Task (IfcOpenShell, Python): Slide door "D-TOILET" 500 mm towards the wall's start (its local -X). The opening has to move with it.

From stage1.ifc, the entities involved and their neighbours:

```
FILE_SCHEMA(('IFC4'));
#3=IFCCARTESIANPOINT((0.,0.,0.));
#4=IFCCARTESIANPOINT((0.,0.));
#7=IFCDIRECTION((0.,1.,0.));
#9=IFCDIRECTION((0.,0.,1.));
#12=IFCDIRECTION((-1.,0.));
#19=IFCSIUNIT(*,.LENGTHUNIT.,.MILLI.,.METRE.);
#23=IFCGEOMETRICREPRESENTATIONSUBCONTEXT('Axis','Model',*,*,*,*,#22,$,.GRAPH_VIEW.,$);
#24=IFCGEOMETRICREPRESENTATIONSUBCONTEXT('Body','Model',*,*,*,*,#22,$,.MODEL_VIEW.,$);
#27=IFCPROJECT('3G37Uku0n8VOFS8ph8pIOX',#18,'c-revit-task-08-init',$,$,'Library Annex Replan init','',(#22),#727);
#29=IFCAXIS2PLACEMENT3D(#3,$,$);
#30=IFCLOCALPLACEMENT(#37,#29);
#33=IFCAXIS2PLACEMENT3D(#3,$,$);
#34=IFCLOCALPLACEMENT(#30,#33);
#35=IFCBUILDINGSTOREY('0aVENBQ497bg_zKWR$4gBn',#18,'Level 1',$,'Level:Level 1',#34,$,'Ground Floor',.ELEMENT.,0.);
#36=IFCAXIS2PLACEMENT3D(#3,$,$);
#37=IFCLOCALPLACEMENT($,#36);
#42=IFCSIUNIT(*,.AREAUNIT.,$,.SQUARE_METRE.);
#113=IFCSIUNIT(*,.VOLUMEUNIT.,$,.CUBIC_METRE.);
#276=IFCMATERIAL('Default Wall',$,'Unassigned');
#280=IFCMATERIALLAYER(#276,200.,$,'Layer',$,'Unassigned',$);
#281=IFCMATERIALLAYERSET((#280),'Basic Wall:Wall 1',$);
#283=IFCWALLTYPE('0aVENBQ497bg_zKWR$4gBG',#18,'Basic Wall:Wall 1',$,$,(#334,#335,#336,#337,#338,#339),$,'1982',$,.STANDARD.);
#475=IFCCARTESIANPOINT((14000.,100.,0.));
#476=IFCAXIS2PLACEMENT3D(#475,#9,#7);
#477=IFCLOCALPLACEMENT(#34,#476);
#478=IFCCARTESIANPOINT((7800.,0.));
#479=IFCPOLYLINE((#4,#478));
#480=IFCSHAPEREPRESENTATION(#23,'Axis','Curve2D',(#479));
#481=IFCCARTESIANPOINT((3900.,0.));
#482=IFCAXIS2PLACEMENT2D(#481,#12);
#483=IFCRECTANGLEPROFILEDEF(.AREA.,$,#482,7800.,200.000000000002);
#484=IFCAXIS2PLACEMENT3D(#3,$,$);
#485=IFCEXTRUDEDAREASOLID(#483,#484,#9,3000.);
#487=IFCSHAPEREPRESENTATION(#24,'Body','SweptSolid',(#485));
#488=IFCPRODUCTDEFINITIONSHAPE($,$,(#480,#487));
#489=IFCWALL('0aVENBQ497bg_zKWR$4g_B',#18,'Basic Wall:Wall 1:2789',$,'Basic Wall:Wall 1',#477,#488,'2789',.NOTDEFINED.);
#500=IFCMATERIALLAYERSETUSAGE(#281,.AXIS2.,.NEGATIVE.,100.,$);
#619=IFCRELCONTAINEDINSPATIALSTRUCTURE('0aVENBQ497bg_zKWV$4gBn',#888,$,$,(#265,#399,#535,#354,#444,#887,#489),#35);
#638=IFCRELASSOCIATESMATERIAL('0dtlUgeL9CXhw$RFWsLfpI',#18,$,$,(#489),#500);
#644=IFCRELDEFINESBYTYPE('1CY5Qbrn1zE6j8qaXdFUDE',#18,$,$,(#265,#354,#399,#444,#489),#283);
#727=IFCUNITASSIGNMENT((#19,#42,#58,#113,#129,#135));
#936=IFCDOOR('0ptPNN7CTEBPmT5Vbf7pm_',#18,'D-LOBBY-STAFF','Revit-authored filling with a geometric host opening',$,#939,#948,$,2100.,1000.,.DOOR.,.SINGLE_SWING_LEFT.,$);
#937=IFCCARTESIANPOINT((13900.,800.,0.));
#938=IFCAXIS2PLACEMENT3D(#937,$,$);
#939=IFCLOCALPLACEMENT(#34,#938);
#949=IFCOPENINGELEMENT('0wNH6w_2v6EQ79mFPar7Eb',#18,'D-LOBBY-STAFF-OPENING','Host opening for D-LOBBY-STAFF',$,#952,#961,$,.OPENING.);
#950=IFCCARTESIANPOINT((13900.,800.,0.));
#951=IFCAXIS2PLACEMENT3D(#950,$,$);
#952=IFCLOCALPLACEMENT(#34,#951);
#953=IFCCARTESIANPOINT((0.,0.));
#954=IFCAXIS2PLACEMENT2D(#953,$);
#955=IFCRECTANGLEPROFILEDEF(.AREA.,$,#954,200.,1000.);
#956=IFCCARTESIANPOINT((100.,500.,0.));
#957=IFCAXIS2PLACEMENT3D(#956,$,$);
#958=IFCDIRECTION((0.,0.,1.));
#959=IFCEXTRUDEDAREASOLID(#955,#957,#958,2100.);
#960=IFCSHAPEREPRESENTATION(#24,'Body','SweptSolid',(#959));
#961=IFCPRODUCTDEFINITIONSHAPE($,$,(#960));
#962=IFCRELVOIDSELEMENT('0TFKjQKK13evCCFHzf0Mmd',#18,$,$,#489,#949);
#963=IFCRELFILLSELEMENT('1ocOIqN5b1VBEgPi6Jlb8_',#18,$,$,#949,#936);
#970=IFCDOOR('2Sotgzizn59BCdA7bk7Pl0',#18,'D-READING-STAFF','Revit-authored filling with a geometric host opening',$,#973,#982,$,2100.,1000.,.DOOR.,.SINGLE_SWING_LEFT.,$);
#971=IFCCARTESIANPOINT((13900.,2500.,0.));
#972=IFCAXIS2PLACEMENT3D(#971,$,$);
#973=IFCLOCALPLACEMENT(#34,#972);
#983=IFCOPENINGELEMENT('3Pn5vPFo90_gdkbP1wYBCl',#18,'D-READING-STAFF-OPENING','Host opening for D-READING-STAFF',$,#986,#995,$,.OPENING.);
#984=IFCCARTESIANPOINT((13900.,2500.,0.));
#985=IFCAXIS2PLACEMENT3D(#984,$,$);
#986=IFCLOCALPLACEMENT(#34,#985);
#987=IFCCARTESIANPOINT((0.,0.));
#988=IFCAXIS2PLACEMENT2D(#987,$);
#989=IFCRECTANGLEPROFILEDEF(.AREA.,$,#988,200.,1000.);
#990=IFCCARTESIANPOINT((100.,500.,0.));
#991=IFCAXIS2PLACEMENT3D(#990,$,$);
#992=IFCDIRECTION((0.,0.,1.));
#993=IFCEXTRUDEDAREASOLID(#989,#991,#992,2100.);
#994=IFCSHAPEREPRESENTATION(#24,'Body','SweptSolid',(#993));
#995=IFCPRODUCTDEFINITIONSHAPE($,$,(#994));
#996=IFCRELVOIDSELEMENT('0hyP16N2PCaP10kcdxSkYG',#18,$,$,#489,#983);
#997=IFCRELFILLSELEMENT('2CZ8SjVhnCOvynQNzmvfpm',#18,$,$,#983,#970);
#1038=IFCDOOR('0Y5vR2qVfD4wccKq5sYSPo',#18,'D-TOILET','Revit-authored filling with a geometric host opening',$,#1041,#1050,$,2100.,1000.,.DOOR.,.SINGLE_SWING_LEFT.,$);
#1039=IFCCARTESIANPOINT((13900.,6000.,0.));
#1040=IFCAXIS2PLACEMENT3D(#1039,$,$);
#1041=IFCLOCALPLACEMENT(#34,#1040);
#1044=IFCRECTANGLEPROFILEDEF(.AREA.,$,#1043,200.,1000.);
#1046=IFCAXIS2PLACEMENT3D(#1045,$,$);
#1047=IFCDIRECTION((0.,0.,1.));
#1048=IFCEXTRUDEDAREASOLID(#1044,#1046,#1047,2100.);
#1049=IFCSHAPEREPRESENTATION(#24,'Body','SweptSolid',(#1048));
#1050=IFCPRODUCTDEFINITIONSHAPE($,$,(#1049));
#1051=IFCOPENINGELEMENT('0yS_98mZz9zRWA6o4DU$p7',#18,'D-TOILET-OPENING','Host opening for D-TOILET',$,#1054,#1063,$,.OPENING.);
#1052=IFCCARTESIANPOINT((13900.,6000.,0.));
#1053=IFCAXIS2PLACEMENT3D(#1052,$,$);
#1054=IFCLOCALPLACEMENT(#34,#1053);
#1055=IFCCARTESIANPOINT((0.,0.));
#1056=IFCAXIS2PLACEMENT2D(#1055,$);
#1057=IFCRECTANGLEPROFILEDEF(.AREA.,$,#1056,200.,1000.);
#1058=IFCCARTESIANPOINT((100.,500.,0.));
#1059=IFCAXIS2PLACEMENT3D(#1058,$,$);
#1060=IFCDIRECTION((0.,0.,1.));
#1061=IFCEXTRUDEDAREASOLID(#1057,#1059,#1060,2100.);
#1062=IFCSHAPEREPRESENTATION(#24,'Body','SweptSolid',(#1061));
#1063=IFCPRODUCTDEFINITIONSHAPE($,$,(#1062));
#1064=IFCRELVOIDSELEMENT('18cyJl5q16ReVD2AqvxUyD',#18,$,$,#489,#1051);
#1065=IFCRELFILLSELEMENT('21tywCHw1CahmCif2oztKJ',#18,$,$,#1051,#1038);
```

```python
import ifcopenshell
import ifcopenshell.api.geometry
import ifcopenshell.util.placement
import ifcopenshell.util.unit

model = ifcopenshell.open("stage1.ifc")
unit_scale = ifcopenshell.util.unit.calculate_unit_scale(model)

door = model.by_guid("0Y5vR2qVfD4wccKq5sYSPo")
opening = door.FillsVoids[0].RelatingOpeningElement
wall = opening.VoidsElements[0].RelatingBuildingElement

wall_matrix = ifcopenshell.util.placement.get_local_placement(wall.ObjectPlacement)
shift = wall_matrix[:3, 0] * -0.5 / unit_scale
before = ifcopenshell.util.placement.get_local_placement(door.ObjectPlacement)[:3, 3].copy()

# The door is not placed relative to its opening, so move both.
for product in (opening, door):
    matrix = ifcopenshell.util.placement.get_local_placement(product.ObjectPlacement)
    matrix[:3, 3] += shift
    ifcopenshell.api.geometry.edit_object_placement(model, product=product, matrix=matrix, is_si=False)

after = ifcopenshell.util.placement.get_local_placement(door.ObjectPlacement)[:3, 3]
print("door moved by", (after - before).round(3) + 0.0)

model.write("stage1_rev.ifc")
```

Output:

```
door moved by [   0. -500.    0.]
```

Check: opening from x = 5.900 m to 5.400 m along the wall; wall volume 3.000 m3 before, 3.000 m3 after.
